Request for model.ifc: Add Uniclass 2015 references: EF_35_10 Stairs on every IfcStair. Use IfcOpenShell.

First a look at what the model holds.

```python
import ifcopenshell

model = ifcopenshell.open("model.ifc")
print(model.schema)
print("classifications:", [c.Name for c in model.by_type("IfcClassification")])
for ifc_class in ("IfcDoor", "IfcRoof", "IfcStair", "IfcWall", "IfcWindow"):
    print(ifc_class, len(model.by_type(ifc_class)))
```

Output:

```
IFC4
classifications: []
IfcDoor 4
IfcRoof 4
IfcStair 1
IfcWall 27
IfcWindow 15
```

```python
import ifcopenshell
import ifcopenshell.api.classification

model = ifcopenshell.open("model.ifc")

system = ifcopenshell.api.classification.add_classification(model, classification="Uniclass 2015")

codes = {
    "IfcStair": ("EF_35_10", "Stairs"),
}
for ifc_class, (code, name) in codes.items():
    products = model.by_type(ifc_class)
    ifcopenshell.api.classification.add_reference(
        model, products=products, classification=system, identification=code, name=name
    )
    print(code, len(products))

model.write("model_updated.ifc")
```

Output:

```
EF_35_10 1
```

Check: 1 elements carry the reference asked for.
